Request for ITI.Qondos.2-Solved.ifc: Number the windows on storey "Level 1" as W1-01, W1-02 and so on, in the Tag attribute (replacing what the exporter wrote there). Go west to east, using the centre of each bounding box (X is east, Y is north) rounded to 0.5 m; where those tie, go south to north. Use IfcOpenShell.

First a look at what the model holds.

```python
import ifcopenshell
import ifcopenshell.util.element
import ifcopenshell.util.placement

model = ifcopenshell.open("ITI.Qondos.2-Solved.ifc")
print(model.schema)
storey = next(s for s in model.by_type("IfcBuildingStorey") if s.Name == "Level 1")
windows = [e for e in ifcopenshell.util.element.get_decomposition(storey) if e.is_a("IfcWindow")]
for e in sorted(windows, key=lambda e: e.id()):
    origin = ifcopenshell.util.placement.get_local_placement(e.ObjectPlacement)[:3, 3]
    print(e.id(), e.Tag, e.Name, origin.round(2) + 0.0, sep=" | ")
```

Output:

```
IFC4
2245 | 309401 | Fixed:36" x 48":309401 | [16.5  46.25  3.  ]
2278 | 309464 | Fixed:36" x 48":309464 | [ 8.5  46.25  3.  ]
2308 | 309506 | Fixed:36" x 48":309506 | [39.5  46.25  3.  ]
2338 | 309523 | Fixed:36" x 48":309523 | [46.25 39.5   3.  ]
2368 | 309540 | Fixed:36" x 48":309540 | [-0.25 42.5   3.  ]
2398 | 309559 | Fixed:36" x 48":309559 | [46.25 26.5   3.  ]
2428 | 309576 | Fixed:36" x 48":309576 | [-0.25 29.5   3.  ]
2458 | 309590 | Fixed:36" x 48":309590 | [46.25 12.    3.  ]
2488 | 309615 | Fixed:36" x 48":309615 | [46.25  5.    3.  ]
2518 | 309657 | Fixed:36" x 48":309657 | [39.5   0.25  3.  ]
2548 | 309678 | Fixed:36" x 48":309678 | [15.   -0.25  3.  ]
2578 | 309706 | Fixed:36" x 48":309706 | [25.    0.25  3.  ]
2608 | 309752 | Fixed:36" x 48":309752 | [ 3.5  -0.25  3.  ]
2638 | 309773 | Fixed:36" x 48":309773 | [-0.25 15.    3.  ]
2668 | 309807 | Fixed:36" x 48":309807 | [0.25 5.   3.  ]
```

```python
import ifcopenshell
import ifcopenshell.geom
import ifcopenshell.util.element
import ifcopenshell.util.shape

model = ifcopenshell.open("ITI.Qondos.2-Solved.ifc")
settings = ifcopenshell.geom.settings()
settings.set("use-world-coords", True)


def centre(element):
    shape = ifcopenshell.geom.create_shape(settings, element)
    return ifcopenshell.util.shape.get_bbox_centroid(shape.geometry)


storey = next(s for s in model.by_type("IfcBuildingStorey") if s.Name == "Level 1")
windows = [e for e in ifcopenshell.util.element.get_decomposition(storey) if e.is_a("IfcWindow")]

# Insertion points can sit at a corner or the storey origin, so sort by the geometry (in metres).
centres = {e: centre(e) for e in windows}
windows.sort(key=lambda e: (round(centres[e][0] / 0.5), centres[e][1]))

for i, e in enumerate(windows, start=1):
    number = f"W1-{i:02d}"
    e.Tag = number
    print(e.id(), number)

model.write("ITI.Qondos.2-Solved_updated.ifc")
```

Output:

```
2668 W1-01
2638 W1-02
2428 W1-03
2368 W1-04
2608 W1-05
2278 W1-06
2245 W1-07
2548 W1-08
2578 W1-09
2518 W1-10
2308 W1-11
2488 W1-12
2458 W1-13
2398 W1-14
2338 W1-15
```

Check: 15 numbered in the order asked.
